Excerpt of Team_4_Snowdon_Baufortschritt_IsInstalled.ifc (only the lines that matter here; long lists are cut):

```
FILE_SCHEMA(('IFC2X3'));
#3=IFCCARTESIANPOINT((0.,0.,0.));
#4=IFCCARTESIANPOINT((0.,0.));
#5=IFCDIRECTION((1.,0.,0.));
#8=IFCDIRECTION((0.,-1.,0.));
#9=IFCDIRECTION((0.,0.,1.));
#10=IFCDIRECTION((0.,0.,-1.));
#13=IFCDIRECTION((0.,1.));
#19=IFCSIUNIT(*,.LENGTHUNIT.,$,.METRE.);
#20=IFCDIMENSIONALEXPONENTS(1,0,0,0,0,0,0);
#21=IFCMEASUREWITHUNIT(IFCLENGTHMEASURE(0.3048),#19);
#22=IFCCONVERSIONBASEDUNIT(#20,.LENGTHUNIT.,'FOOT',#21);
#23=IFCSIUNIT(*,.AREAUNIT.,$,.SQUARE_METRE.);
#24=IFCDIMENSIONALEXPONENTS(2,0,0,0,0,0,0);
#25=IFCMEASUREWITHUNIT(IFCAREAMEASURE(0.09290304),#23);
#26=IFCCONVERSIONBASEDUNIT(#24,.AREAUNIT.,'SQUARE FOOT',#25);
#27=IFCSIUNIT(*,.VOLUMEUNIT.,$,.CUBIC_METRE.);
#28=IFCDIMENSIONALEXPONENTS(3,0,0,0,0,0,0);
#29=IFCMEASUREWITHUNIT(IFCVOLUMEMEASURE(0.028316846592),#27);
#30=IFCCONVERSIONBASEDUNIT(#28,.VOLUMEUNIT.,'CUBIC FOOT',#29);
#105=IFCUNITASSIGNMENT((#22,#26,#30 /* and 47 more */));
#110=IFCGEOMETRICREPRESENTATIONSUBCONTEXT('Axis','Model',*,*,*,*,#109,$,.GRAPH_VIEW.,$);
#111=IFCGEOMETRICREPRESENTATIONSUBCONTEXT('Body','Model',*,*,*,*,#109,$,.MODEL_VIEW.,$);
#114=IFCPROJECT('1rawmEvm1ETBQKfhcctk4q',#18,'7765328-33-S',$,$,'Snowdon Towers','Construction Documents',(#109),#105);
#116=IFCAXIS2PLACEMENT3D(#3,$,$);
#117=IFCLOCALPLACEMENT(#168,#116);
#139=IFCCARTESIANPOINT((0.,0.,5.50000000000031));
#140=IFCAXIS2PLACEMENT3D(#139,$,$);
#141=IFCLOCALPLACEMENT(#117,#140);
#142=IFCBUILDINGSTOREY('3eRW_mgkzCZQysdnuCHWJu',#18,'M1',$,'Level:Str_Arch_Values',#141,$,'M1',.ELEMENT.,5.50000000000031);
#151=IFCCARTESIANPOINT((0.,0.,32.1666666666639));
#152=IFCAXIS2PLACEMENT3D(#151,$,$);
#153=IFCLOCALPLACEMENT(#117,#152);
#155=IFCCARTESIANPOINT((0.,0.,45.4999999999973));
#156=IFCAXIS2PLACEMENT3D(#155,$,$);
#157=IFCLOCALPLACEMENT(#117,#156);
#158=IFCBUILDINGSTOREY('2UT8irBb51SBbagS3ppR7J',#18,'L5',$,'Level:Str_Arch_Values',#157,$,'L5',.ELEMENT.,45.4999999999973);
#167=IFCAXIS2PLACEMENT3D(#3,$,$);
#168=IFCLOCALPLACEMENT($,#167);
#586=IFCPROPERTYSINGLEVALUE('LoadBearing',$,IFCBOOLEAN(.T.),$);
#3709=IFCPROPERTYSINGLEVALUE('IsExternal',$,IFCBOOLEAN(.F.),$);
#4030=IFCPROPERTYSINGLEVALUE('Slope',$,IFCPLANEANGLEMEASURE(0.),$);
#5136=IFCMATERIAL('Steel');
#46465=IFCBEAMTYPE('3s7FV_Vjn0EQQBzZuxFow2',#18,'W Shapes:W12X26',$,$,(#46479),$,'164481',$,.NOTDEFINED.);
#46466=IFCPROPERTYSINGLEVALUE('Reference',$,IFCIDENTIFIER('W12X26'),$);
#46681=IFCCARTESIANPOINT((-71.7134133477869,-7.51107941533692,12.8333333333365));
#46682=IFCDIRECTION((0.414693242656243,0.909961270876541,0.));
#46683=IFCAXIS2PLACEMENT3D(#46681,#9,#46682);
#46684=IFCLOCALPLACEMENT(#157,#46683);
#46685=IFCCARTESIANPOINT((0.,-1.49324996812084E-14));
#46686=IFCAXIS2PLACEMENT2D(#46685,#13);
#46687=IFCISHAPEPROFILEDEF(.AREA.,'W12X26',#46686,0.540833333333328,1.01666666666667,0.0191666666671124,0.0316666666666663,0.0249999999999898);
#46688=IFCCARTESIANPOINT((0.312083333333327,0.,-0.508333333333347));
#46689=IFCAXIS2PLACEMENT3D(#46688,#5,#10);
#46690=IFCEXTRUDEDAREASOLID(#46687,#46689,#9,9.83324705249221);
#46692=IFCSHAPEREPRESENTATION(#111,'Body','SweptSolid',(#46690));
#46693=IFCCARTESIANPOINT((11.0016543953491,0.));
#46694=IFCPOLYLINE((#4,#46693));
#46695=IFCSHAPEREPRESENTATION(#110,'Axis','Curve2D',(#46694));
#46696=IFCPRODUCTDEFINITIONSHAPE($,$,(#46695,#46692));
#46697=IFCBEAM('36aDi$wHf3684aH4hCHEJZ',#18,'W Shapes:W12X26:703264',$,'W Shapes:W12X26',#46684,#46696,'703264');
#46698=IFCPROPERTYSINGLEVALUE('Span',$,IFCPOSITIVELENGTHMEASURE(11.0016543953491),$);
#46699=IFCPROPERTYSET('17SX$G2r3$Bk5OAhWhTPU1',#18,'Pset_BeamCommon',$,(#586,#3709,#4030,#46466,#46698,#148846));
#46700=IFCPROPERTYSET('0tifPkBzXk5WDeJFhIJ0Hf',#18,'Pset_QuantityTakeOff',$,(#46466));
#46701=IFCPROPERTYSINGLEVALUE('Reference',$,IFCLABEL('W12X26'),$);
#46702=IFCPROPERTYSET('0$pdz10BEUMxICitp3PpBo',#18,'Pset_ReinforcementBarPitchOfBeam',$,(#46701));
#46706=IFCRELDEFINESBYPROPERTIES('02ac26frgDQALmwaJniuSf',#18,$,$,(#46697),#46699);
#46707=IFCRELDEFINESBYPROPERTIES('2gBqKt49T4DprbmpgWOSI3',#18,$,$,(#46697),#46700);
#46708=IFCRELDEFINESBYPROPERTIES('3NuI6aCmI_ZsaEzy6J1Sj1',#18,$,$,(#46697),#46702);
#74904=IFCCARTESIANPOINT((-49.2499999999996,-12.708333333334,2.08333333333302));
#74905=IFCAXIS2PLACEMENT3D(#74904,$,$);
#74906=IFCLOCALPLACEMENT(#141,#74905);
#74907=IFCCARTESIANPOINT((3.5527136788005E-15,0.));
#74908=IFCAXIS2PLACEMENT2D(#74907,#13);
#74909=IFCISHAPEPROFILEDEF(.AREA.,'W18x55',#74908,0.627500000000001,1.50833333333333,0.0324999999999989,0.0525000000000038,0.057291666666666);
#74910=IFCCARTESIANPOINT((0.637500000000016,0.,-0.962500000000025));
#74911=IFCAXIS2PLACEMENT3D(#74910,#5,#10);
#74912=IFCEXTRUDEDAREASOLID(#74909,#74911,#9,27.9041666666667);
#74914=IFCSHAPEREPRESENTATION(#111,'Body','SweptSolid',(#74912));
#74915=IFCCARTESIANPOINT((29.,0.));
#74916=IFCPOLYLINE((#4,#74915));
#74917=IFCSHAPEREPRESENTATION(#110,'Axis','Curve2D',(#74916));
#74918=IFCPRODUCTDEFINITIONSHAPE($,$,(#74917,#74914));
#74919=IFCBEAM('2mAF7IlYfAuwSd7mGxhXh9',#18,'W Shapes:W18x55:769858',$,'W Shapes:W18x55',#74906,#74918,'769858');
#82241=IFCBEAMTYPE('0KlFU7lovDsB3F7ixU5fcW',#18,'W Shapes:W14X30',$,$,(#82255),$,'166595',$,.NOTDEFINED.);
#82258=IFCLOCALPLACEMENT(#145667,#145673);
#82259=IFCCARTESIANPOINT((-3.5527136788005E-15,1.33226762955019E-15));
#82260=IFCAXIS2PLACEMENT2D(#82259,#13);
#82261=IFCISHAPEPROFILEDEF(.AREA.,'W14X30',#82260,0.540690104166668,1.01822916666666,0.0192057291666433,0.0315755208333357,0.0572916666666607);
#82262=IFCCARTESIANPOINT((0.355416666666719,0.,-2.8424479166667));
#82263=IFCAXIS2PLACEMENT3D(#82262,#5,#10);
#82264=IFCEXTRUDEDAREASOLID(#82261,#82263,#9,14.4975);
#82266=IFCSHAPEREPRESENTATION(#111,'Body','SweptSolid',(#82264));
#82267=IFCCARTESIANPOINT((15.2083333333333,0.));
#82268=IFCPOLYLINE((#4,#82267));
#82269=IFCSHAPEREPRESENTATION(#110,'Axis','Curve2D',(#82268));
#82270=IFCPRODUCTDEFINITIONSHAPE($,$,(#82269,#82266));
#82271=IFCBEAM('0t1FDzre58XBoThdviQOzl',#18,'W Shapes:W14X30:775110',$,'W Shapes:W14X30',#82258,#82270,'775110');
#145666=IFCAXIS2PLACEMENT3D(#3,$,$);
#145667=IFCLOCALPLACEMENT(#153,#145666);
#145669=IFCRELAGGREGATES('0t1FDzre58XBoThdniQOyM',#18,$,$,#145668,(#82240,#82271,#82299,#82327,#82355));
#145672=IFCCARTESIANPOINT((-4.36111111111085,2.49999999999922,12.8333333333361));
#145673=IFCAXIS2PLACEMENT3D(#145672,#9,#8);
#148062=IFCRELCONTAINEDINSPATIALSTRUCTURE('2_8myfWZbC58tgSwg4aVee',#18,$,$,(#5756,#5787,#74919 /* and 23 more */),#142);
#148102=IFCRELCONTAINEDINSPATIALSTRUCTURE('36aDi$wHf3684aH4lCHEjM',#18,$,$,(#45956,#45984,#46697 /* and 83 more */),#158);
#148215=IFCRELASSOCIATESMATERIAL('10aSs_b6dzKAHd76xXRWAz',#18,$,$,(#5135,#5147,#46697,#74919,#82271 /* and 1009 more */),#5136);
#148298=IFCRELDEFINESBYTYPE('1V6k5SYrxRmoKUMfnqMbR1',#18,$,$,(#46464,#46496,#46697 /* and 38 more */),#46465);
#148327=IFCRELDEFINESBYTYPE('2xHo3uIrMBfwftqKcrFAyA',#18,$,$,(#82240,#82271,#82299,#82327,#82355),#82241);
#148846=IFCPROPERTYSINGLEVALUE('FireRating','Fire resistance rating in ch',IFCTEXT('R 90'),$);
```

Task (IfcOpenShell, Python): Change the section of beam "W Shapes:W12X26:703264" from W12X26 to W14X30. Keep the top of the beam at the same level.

```python
import ifcopenshell
import ifcopenshell.api.pset
import ifcopenshell.api.type
import ifcopenshell.util.element
import ifcopenshell.util.representation

model = ifcopenshell.open("Team_4_Snowdon_Baufortschritt_IsInstalled.ifc")

member = model.by_guid("36aDi$wHf3684aH4hCHEJZ")
source = next(p for p in model.by_type("IfcIShapeProfileDef") if p.ProfileName == "W14X30")

body = ifcopenshell.util.representation.get_representation(member, "Model", "Body")
solid = body.Items[0]
old_profile = solid.SweptArea

# Copy the section's sizes but keep this member's own profile position.
profile = ifcopenshell.util.element.copy(model, source)
# Profiles are centred, so shift by half the change in depth to hold the top.
shift = (old_profile.OverallDepth - profile.OverallDepth) / 2
x, y = old_profile.Position.Location.Coordinates
up = (-1.0, 0.0)  # upwards, in the solid's own plane
location = model.createIfcCartesianPoint((x + up[0] * shift, y + up[1] * shift))
profile.Position = model.createIfcAxis2Placement2D(location, old_profile.Position.RefDirection)
solid.SweptArea = profile
if not model.get_total_inverses(old_profile):
    ifcopenshell.util.element.remove_deep2(model, old_profile)

new_type = model.by_id(82241)
ifcopenshell.api.type.assign_type(
    model, related_objects=[member], relating_type=new_type, should_map_representations=False
)
member.Name = member.Name.replace("W12X26", "W14X30")
member.ObjectType = "W Shapes:W14X30"
pset = model.by_id(ifcopenshell.util.element.get_pset(member, "Pset_BeamCommon", should_inherit=False)["id"])
ifcopenshell.api.pset.edit_pset(model, pset=pset, properties={"Reference": "W14X30"})
pset = model.by_id(ifcopenshell.util.element.get_pset(member, "Pset_QuantityTakeOff", should_inherit=False)["id"])
ifcopenshell.api.pset.edit_pset(model, pset=pset, properties={"Reference": "W14X30"})
pset = model.by_id(ifcopenshell.util.element.get_pset(member, "Pset_ReinforcementBarPitchOfBeam", should_inherit=False)["id"])
ifcopenshell.api.pset.edit_pset(model, pset=pset, properties={"Reference": "W14X30"})

print(solid.SweptArea)

model.write("Team_4_Snowdon_Baufortschritt_IsInstalled_edited.ifc")
```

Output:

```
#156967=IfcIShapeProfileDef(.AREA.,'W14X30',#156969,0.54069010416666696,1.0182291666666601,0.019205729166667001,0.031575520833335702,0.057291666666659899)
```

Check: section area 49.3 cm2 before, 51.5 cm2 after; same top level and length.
